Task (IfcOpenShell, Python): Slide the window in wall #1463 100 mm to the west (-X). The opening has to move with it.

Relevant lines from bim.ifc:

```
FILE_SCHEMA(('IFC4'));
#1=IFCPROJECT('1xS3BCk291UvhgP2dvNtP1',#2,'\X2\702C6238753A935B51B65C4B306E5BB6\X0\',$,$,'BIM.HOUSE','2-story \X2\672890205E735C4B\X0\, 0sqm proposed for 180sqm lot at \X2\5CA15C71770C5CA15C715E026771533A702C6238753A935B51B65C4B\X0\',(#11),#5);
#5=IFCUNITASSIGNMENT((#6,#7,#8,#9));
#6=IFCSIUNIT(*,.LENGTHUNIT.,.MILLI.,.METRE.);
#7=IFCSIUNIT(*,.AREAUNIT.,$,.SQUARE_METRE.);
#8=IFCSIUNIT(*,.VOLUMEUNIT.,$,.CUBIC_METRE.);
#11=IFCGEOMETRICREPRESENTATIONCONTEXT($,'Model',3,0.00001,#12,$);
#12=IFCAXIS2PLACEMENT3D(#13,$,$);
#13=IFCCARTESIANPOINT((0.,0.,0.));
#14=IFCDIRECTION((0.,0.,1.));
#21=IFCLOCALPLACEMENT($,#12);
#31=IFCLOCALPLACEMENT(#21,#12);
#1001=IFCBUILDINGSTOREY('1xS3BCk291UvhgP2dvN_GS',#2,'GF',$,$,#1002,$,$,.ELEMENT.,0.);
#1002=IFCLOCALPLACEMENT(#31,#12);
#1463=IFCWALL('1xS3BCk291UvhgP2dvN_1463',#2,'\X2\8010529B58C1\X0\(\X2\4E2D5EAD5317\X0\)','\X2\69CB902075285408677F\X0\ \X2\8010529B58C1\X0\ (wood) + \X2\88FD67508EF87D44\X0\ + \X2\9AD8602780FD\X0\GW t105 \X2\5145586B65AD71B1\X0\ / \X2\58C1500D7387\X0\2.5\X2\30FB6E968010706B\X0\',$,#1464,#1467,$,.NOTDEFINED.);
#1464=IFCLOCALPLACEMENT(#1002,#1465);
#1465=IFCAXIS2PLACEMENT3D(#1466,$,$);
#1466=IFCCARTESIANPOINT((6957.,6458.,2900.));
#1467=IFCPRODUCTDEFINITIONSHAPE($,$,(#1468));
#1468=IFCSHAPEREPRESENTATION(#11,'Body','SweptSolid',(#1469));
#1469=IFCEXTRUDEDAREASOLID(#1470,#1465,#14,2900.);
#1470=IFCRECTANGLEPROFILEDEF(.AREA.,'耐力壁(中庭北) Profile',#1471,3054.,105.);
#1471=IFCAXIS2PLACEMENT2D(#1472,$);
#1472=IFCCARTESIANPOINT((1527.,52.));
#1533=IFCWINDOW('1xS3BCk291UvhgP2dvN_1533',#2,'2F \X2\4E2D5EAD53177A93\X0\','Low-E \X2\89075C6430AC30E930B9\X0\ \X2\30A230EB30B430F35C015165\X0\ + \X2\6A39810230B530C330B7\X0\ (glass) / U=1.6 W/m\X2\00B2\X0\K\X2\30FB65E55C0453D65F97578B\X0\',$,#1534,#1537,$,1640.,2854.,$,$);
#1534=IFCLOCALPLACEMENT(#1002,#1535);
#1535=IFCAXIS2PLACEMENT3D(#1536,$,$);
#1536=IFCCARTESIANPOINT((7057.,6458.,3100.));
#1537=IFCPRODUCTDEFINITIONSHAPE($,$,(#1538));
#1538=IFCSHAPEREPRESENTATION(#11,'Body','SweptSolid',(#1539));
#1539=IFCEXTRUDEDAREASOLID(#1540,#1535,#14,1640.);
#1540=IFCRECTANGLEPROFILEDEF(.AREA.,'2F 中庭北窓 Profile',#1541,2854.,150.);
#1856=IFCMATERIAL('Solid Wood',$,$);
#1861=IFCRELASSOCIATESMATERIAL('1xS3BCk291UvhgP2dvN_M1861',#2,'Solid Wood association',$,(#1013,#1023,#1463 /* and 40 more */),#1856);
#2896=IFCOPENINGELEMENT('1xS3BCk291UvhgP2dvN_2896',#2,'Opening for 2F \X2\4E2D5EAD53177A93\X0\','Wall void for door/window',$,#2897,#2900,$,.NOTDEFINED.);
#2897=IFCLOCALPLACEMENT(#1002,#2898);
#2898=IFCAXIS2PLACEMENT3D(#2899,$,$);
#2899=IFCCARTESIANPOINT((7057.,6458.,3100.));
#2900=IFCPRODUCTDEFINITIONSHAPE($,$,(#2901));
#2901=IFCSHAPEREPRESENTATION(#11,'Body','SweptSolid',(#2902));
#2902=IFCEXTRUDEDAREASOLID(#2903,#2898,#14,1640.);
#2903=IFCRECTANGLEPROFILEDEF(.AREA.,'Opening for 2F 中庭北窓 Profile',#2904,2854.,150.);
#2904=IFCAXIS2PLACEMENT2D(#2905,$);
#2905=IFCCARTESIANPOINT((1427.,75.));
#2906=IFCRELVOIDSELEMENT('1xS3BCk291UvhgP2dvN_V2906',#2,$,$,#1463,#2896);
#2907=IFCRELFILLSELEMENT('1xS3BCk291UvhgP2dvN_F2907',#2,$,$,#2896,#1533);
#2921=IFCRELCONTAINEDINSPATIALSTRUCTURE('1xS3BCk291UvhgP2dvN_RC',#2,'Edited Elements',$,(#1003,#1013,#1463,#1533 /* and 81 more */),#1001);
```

```python
import ifcopenshell
import ifcopenshell.api.geometry
import ifcopenshell.util.placement
import ifcopenshell.util.unit

model = ifcopenshell.open("bim.ifc")
unit_scale = ifcopenshell.util.unit.calculate_unit_scale(model)

window = model.by_guid("1xS3BCk291UvhgP2dvN_1533")
opening = window.FillsVoids[0].RelatingOpeningElement
wall = opening.VoidsElements[0].RelatingBuildingElement

wall_matrix = ifcopenshell.util.placement.get_local_placement(wall.ObjectPlacement)
shift = wall_matrix[:3, 0] * -0.1 / unit_scale
before = ifcopenshell.util.placement.get_local_placement(window.ObjectPlacement)[:3, 3].copy()

# The window is not placed relative to its opening, so move both.
for product in (opening, window):
    matrix = ifcopenshell.util.placement.get_local_placement(product.ObjectPlacement)
    matrix[:3, 3] += shift
    ifcopenshell.api.geometry.edit_object_placement(model, product=product, matrix=matrix, is_si=False)

after = ifcopenshell.util.placement.get_local_placement(window.ObjectPlacement)[:3, 3]
print("window moved by", (after - before).round(3) + 0.0)

model.write("bim_updated.ifc")
```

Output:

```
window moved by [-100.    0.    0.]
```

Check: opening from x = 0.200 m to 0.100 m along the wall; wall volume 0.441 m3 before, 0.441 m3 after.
